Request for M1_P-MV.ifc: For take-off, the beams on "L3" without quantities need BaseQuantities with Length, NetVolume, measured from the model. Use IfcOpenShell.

First a look at what the model holds.

```python
import ifcopenshell
import ifcopenshell.util.element
import ifcopenshell.util.unit

model = ifcopenshell.open("M1_P-MV.ifc")
print(model.schema)
for unit_type in ("LENGTHUNIT", "AREAUNIT", "VOLUMEUNIT"):
    print(unit_type, ifcopenshell.util.unit.calculate_unit_scale(model, unit_type))
storey = next(s for s in model.by_type("IfcBuildingStorey") if s.Name == "L3")
beams = [e for e in ifcopenshell.util.element.get_decomposition(storey) if e.is_a("IfcBeam")]
for e in sorted(beams, key=lambda e: e.id()):
    print(e.id(), e.is_a(), e.Name, list(ifcopenshell.util.element.get_psets(e, qtos_only=True)), sep=" | ")
```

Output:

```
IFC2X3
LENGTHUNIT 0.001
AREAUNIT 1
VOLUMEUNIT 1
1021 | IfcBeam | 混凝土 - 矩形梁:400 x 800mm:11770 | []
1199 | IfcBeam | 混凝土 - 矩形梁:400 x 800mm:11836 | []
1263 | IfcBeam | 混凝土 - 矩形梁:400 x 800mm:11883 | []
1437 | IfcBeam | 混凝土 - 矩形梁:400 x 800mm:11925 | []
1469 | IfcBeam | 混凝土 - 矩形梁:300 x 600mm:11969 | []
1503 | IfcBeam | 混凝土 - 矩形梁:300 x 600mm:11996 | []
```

```python
import ifcopenshell
import ifcopenshell.api.pset
import ifcopenshell.geom
import ifcopenshell.util.element
import ifcopenshell.util.shape
import ifcopenshell.util.unit

model = ifcopenshell.open("M1_P-MV.ifc")
unit_scale = ifcopenshell.util.unit.calculate_unit_scale(model)
volume_scale = ifcopenshell.util.unit.calculate_unit_scale(model, "VOLUMEUNIT")
settings = ifcopenshell.geom.settings()

storey = next(s for s in model.by_type("IfcBuildingStorey") if s.Name == "L3")
beams = [e for e in ifcopenshell.util.element.get_decomposition(storey) if e.is_a("IfcBeam")]

for e in sorted(beams, key=lambda e: e.id()):
    if ifcopenshell.util.element.get_psets(e, qtos_only=True, should_inherit=False):
        continue
    # Geometry comes back in metres, in the element's own axes.
    shape = ifcopenshell.geom.create_shape(settings, e)
    values = {
        "Length": ifcopenshell.util.shape.get_max_xyz(shape.geometry) / unit_scale,
        "NetVolume": ifcopenshell.util.shape.get_volume(shape.geometry) / volume_scale,
    }
    qto = ifcopenshell.api.pset.add_qto(model, product=e, name="BaseQuantities")
    ifcopenshell.api.pset.edit_qto(model, qto=qto, properties=values)
    print(e.id(), {k: round(v, 3) for k, v in values.items()})

model.write("M1_P-MV_rev.ifc")
```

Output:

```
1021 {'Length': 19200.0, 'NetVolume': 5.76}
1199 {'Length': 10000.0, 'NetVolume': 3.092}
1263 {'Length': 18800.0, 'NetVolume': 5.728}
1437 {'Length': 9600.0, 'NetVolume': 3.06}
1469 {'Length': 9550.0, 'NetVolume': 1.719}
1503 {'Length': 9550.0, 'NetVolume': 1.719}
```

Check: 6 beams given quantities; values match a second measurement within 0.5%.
